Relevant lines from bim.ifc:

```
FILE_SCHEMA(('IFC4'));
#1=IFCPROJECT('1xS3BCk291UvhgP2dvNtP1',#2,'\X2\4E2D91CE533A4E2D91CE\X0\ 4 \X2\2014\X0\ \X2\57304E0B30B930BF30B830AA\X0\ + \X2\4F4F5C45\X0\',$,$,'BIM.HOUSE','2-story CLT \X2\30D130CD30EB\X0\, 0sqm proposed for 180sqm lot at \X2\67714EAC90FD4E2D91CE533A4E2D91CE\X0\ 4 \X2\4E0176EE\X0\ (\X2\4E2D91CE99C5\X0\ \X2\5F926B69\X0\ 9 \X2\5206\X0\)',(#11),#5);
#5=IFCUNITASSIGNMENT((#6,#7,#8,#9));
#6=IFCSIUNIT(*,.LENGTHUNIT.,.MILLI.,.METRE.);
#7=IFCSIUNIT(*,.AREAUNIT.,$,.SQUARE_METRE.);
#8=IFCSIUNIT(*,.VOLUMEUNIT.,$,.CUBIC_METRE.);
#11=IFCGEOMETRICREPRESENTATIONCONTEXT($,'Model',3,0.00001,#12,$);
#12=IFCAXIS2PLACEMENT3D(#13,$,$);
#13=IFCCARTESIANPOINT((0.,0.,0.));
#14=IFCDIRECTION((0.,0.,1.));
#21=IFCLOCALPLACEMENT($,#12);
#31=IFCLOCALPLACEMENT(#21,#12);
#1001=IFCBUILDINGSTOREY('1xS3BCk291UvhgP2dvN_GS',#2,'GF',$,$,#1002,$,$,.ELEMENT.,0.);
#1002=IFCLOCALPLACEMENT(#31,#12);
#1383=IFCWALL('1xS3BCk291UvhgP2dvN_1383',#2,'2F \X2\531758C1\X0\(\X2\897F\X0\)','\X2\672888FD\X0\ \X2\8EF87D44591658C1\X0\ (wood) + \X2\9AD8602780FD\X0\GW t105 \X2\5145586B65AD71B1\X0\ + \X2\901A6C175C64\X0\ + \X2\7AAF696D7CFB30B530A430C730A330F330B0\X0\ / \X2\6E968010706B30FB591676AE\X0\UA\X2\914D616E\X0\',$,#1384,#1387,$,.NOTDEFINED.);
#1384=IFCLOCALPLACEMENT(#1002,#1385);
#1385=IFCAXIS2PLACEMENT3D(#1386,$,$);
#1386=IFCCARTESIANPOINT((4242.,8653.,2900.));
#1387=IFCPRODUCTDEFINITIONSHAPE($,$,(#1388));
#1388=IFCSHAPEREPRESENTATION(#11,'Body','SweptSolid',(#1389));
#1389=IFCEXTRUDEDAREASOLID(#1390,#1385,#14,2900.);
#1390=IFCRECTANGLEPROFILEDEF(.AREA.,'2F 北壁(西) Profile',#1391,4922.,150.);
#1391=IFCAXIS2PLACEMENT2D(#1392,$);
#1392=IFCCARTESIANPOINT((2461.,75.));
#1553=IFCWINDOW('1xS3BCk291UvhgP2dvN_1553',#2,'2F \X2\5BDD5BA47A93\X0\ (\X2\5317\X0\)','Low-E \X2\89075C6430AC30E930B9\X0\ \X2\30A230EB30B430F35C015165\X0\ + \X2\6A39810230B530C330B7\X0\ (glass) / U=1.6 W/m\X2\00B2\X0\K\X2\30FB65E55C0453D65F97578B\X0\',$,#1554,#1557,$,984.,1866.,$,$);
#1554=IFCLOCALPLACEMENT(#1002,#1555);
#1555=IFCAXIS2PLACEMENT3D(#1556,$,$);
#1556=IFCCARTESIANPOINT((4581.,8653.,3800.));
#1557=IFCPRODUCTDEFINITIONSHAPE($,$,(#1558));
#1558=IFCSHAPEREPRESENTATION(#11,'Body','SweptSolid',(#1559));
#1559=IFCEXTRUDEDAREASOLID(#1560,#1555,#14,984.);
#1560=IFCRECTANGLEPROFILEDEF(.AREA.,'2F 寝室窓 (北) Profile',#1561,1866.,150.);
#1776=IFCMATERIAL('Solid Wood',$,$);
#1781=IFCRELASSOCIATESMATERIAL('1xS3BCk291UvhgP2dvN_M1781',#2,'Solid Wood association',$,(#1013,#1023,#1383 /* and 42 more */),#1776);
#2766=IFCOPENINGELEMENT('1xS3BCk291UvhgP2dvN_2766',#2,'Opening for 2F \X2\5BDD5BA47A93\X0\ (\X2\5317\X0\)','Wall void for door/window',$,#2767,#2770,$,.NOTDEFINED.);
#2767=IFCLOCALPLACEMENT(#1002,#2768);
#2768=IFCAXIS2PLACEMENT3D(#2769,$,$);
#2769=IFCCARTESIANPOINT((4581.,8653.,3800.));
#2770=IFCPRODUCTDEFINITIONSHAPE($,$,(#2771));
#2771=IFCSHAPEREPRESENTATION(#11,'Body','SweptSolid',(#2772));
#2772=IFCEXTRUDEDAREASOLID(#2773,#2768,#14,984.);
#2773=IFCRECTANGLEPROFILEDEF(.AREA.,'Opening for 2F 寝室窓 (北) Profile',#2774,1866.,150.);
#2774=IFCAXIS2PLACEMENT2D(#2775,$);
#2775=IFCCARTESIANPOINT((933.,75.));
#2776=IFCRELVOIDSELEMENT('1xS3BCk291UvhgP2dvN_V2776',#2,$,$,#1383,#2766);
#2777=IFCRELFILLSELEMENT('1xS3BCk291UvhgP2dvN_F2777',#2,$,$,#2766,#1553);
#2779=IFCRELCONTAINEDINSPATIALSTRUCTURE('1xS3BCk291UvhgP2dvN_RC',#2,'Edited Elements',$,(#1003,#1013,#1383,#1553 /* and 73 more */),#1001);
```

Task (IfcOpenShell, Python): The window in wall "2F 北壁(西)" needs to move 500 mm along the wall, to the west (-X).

```python
import ifcopenshell
import ifcopenshell.api.geometry
import ifcopenshell.util.placement
import ifcopenshell.util.unit

model = ifcopenshell.open("bim.ifc")
unit_scale = ifcopenshell.util.unit.calculate_unit_scale(model)

window = model.by_guid("1xS3BCk291UvhgP2dvN_1553")
opening = window.FillsVoids[0].RelatingOpeningElement
wall = opening.VoidsElements[0].RelatingBuildingElement

wall_matrix = ifcopenshell.util.placement.get_local_placement(wall.ObjectPlacement)
shift = wall_matrix[:3, 0] * -0.5 / unit_scale
before = ifcopenshell.util.placement.get_local_placement(window.ObjectPlacement)[:3, 3].copy()

# The window is not placed relative to its opening, so move both.
for product in (opening, window):
    matrix = ifcopenshell.util.placement.get_local_placement(product.ObjectPlacement)
    matrix[:3, 3] += shift
    ifcopenshell.api.geometry.edit_object_placement(model, product=product, matrix=matrix, is_si=False)

after = ifcopenshell.util.placement.get_local_placement(window.ObjectPlacement)[:3, 3]
print("window moved by", (after - before).round(3) + 0.0)

model.write("bim-out.ifc")
```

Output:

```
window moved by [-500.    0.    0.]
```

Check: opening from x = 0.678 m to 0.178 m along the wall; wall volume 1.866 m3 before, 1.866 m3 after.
